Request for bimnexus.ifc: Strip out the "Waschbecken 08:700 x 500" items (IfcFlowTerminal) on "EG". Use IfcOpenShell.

First a look at what the model holds.

```python
import ifcopenshell
import ifcopenshell.util.element

model = ifcopenshell.open("bimnexus.ifc")
print(model.schema)
storey = next(s for s in model.by_type("IfcBuildingStorey") if s.Name == "EG")
terminals = [e for e in ifcopenshell.util.element.get_decomposition(storey) if e.is_a("IfcFlowTerminal")]
seen = {}
for e in terminals:
    element_type = ifcopenshell.util.element.get_type(e)
    name = element_type.Name if element_type not in (None, e) else None
    seen[name] = seen.get(name, 0) + 1
for name, count in sorted(seen.items(), key=str):
    print(count, "x", name)
```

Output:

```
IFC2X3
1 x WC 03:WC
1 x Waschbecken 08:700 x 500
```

```python
import ifcopenshell
import ifcopenshell.api.root
import ifcopenshell.util.element

model = ifcopenshell.open("bimnexus.ifc")

storey = next(s for s in model.by_type("IfcBuildingStorey") if s.Name == "EG")
terminals = [e for e in ifcopenshell.util.element.get_decomposition(storey) if e.is_a("IfcFlowTerminal")]
targets = [e for e in terminals if (t := ifcopenshell.util.element.get_type(e)) not in (None, e) and t.Name == "Waschbecken 08:700 x 500"]

for e in targets:
    ifcopenshell.api.root.remove_product(model, product=e)
print(len(targets), "removed")

model.write("bimnexus_edited.ifc")
```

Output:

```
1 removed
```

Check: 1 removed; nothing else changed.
